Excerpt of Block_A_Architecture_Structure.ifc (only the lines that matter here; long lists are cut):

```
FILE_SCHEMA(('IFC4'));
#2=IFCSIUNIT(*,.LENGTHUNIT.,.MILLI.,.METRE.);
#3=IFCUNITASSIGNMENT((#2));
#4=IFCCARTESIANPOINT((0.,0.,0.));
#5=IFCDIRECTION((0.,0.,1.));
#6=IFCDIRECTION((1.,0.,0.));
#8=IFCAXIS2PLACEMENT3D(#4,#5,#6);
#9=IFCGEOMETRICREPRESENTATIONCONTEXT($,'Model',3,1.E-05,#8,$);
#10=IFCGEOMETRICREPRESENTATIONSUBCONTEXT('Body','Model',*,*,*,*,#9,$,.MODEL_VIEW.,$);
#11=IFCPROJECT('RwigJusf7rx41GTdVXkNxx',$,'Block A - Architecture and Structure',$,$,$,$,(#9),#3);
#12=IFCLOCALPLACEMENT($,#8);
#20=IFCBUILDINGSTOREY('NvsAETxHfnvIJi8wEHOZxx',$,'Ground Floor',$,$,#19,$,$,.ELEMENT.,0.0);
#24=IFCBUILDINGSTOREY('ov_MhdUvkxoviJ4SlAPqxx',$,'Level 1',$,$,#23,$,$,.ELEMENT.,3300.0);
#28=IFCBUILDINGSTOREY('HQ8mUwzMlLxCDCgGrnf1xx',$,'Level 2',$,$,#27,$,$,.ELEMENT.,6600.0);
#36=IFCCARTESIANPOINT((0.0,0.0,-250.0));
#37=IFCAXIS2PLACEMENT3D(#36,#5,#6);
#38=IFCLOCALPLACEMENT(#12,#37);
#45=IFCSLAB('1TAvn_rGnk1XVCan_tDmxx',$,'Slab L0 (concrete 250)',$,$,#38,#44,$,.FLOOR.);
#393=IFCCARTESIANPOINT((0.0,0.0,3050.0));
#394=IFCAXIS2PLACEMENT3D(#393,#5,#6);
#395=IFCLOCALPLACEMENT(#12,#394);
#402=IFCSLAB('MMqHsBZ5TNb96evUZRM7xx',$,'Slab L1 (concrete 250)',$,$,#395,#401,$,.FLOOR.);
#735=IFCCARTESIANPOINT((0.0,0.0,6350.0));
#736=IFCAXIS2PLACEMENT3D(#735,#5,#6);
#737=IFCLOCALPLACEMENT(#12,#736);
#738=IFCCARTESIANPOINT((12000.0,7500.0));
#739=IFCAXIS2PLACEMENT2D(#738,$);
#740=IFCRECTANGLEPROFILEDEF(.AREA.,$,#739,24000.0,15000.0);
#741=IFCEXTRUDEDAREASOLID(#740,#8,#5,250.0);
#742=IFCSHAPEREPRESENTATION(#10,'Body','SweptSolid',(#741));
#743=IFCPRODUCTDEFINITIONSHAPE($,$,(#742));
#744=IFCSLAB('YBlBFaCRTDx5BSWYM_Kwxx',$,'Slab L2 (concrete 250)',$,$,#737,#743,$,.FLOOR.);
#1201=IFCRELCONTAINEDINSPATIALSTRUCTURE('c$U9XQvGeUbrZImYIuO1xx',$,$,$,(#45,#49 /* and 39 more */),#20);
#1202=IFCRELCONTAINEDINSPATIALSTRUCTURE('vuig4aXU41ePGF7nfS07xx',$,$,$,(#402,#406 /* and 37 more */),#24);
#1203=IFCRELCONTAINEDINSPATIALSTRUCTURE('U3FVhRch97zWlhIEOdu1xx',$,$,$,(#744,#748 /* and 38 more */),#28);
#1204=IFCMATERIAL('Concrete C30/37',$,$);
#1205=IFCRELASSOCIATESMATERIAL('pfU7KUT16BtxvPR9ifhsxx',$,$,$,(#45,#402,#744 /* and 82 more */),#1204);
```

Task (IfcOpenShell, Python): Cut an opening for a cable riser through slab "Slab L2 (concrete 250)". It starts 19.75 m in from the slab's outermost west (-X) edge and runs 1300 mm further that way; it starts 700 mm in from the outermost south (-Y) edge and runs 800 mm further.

```python
import numpy as np
import ifcopenshell
import ifcopenshell.api.feature
import ifcopenshell.api.geometry
import ifcopenshell.api.root
import ifcopenshell.geom
import ifcopenshell.util.placement
import ifcopenshell.util.representation
import ifcopenshell.util.shape
import ifcopenshell.util.unit

model = ifcopenshell.open("Block_A_Architecture_Structure.ifc")
unit_scale = ifcopenshell.util.unit.calculate_unit_scale(model)
settings = ifcopenshell.geom.settings()


def volume(element):
    """Net volume in cubic metres, openings subtracted."""
    shape = ifcopenshell.geom.create_shape(settings, element)
    return ifcopenshell.util.shape.get_volume(shape.geometry)


slab = model.by_id(744)
before = volume(slab)

# Extent in the slab's own axes, in metres. The edges named are its -X and -Y sides.
slab_shape = ifcopenshell.geom.create_shape(settings, slab)
vertices = ifcopenshell.util.shape.get_vertices(slab_shape.geometry)
x_min, y_min, bottom = vertices.min(axis=0)
top = vertices[:, 2].max()

opening = ifcopenshell.api.root.create_entity(model, ifc_class="IfcOpeningElement", name="Cable riser opening", predefined_type="OPENING")
context = ifcopenshell.util.representation.get_context(model, "Model", "Body", "MODEL_VIEW")
width, depth = 1.3, 0.8
outline = [(0.0, 0.0), (width, 0.0), (width, depth), (0.0, depth), (0.0, 0.0)]
# Overshoot both faces by 50 mm so the cut is clean.
shape = ifcopenshell.api.geometry.add_slab_representation(
    model, context=context, depth=top - bottom + 0.1, polyline=outline
)
ifcopenshell.api.geometry.assign_representation(model, product=opening, representation=shape)

matrix = ifcopenshell.util.placement.get_local_placement(slab.ObjectPlacement)
matrix[:, 3] = matrix @ np.append(np.array([x_min + 19.75, y_min + 0.7, bottom - 0.05]) / unit_scale, 1.0)
ifcopenshell.api.geometry.edit_object_placement(model, product=opening, matrix=matrix, is_si=False)
ifcopenshell.api.feature.add_feature(model, feature=opening, element=slab)

after = volume(slab)

print(f"slab volume {before:.3f} -> {after:.3f} m3")

model.write("Block_A_Architecture_Structure_updated.ifc")
```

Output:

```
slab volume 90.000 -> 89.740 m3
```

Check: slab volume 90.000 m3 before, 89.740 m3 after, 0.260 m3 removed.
